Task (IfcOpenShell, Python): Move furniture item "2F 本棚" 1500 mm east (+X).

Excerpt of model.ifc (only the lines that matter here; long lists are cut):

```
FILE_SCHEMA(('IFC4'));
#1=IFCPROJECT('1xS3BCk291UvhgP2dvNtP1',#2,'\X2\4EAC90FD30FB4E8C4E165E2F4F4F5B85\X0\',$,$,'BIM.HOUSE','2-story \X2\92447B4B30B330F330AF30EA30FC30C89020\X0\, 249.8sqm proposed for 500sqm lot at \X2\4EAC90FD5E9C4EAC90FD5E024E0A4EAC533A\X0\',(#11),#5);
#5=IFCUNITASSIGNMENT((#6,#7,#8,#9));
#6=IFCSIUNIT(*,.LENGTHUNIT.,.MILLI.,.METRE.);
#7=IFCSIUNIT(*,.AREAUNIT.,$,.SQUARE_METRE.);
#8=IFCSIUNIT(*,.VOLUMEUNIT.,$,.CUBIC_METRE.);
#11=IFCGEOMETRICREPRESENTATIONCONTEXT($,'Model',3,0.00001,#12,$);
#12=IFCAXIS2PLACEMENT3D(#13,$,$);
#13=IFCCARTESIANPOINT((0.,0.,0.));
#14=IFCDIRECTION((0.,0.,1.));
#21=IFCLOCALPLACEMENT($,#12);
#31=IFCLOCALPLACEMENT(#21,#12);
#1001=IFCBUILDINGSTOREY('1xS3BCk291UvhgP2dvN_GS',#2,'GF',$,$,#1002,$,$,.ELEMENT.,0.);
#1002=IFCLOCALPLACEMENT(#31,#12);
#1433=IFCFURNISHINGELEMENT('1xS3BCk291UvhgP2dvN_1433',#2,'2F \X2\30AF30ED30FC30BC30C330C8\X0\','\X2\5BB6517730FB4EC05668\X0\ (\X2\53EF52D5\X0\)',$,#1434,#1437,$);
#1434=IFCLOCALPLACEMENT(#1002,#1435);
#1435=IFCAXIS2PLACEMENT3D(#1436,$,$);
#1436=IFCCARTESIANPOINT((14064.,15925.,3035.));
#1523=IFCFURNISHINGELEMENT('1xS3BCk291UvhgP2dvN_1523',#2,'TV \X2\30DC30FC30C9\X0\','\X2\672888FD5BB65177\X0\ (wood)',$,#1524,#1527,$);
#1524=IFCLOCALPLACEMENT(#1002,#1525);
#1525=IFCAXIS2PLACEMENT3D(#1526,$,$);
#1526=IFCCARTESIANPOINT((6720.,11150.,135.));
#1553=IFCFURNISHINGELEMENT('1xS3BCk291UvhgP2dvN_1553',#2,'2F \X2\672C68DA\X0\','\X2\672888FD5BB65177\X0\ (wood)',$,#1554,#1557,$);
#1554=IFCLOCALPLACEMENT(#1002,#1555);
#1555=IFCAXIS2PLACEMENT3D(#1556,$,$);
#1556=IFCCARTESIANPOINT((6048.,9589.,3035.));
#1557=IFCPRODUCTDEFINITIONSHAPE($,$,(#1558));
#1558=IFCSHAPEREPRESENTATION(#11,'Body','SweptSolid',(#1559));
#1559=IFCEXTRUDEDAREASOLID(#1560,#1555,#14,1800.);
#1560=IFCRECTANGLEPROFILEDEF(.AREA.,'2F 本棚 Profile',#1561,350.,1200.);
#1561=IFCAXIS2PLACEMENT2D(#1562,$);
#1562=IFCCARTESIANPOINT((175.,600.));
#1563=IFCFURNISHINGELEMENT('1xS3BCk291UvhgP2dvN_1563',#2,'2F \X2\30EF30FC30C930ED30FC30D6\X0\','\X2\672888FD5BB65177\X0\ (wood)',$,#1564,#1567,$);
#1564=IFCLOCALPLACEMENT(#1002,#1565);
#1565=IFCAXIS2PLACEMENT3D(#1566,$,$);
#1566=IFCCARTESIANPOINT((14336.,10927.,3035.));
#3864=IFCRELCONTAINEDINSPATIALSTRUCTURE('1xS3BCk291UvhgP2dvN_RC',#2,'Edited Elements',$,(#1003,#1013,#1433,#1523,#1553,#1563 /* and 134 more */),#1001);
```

```python
import ifcopenshell
import ifcopenshell.api.geometry
import ifcopenshell.util.placement

model = ifcopenshell.open("model.ifc")

item = model.by_guid("1xS3BCk291UvhgP2dvN_1553")
matrix = ifcopenshell.util.placement.get_local_placement(item.ObjectPlacement)
matrix[0, 3] += 1500.0
ifcopenshell.api.geometry.edit_object_placement(model, product=item, matrix=matrix, is_si=False)

print(ifcopenshell.util.placement.get_local_placement(item.ObjectPlacement).round(3) + 0.0)

model.write("model_edited.ifc")
```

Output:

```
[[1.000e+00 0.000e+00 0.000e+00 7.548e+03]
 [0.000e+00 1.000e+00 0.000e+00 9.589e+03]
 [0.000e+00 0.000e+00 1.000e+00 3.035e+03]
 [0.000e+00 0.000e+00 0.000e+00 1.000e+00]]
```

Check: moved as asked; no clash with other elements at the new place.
